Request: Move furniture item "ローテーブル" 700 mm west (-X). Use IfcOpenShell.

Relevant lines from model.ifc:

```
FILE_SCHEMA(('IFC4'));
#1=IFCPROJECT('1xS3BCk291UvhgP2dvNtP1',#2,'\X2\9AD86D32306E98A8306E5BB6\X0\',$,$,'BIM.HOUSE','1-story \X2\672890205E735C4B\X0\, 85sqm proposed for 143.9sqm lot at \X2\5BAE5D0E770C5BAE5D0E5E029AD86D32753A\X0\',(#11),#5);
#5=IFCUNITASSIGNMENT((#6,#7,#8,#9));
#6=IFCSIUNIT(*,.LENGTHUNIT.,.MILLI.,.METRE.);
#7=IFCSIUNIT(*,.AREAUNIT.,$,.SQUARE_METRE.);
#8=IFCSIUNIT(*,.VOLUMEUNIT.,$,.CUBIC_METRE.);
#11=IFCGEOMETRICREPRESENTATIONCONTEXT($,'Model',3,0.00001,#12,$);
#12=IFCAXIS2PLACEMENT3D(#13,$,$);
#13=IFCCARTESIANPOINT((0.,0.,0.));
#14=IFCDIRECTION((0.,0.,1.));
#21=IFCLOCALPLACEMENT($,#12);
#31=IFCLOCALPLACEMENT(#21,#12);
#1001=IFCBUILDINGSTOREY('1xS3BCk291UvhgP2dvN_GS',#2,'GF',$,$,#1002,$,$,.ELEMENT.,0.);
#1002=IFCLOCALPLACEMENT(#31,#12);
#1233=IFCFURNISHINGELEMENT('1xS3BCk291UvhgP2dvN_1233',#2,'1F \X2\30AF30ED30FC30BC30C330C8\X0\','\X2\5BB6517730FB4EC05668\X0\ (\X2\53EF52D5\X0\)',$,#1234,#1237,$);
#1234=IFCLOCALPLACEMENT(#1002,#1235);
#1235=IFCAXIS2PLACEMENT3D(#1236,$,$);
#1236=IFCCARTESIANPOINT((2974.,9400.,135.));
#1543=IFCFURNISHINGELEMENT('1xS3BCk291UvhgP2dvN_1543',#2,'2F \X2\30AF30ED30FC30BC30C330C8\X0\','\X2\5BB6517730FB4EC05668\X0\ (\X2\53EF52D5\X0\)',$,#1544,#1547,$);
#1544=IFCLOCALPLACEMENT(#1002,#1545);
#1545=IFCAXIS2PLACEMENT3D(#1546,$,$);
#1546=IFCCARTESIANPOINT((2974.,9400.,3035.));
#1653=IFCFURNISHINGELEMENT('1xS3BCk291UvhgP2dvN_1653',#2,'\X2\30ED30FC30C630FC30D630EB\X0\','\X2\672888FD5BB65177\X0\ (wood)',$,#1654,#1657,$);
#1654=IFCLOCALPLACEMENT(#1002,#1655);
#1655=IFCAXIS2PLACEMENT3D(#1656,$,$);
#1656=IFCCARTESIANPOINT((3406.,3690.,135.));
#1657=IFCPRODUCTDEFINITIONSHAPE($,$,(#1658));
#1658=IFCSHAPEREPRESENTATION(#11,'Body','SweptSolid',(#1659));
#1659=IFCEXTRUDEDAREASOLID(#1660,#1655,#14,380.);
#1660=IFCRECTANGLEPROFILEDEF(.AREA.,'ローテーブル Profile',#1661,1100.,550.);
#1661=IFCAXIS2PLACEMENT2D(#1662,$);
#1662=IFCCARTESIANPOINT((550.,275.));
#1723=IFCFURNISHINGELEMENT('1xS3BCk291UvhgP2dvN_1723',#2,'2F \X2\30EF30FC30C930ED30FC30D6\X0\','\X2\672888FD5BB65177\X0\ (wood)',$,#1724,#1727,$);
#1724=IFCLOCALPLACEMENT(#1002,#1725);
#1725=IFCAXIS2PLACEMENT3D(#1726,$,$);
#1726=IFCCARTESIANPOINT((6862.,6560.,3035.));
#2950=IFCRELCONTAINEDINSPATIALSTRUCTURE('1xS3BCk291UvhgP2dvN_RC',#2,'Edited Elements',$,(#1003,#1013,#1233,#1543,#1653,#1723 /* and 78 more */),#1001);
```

```python
import ifcopenshell
import ifcopenshell.api.geometry
import ifcopenshell.util.placement
import ifcopenshell.util.unit

model = ifcopenshell.open("model.ifc")
unit_scale = ifcopenshell.util.unit.calculate_unit_scale(model)

item = model.by_guid("1xS3BCk291UvhgP2dvN_1653")
matrix = ifcopenshell.util.placement.get_local_placement(item.ObjectPlacement)
matrix[0, 3] -= 0.7 / unit_scale
ifcopenshell.api.geometry.edit_object_placement(model, product=item, matrix=matrix, is_si=False)

print(ifcopenshell.util.placement.get_local_placement(item.ObjectPlacement).round(3) + 0.0)

model.write("model_rev.ifc")
```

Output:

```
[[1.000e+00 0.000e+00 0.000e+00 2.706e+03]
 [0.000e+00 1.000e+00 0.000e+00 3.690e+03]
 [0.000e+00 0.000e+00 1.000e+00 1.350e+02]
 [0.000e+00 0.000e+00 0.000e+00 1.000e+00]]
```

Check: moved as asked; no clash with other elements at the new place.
